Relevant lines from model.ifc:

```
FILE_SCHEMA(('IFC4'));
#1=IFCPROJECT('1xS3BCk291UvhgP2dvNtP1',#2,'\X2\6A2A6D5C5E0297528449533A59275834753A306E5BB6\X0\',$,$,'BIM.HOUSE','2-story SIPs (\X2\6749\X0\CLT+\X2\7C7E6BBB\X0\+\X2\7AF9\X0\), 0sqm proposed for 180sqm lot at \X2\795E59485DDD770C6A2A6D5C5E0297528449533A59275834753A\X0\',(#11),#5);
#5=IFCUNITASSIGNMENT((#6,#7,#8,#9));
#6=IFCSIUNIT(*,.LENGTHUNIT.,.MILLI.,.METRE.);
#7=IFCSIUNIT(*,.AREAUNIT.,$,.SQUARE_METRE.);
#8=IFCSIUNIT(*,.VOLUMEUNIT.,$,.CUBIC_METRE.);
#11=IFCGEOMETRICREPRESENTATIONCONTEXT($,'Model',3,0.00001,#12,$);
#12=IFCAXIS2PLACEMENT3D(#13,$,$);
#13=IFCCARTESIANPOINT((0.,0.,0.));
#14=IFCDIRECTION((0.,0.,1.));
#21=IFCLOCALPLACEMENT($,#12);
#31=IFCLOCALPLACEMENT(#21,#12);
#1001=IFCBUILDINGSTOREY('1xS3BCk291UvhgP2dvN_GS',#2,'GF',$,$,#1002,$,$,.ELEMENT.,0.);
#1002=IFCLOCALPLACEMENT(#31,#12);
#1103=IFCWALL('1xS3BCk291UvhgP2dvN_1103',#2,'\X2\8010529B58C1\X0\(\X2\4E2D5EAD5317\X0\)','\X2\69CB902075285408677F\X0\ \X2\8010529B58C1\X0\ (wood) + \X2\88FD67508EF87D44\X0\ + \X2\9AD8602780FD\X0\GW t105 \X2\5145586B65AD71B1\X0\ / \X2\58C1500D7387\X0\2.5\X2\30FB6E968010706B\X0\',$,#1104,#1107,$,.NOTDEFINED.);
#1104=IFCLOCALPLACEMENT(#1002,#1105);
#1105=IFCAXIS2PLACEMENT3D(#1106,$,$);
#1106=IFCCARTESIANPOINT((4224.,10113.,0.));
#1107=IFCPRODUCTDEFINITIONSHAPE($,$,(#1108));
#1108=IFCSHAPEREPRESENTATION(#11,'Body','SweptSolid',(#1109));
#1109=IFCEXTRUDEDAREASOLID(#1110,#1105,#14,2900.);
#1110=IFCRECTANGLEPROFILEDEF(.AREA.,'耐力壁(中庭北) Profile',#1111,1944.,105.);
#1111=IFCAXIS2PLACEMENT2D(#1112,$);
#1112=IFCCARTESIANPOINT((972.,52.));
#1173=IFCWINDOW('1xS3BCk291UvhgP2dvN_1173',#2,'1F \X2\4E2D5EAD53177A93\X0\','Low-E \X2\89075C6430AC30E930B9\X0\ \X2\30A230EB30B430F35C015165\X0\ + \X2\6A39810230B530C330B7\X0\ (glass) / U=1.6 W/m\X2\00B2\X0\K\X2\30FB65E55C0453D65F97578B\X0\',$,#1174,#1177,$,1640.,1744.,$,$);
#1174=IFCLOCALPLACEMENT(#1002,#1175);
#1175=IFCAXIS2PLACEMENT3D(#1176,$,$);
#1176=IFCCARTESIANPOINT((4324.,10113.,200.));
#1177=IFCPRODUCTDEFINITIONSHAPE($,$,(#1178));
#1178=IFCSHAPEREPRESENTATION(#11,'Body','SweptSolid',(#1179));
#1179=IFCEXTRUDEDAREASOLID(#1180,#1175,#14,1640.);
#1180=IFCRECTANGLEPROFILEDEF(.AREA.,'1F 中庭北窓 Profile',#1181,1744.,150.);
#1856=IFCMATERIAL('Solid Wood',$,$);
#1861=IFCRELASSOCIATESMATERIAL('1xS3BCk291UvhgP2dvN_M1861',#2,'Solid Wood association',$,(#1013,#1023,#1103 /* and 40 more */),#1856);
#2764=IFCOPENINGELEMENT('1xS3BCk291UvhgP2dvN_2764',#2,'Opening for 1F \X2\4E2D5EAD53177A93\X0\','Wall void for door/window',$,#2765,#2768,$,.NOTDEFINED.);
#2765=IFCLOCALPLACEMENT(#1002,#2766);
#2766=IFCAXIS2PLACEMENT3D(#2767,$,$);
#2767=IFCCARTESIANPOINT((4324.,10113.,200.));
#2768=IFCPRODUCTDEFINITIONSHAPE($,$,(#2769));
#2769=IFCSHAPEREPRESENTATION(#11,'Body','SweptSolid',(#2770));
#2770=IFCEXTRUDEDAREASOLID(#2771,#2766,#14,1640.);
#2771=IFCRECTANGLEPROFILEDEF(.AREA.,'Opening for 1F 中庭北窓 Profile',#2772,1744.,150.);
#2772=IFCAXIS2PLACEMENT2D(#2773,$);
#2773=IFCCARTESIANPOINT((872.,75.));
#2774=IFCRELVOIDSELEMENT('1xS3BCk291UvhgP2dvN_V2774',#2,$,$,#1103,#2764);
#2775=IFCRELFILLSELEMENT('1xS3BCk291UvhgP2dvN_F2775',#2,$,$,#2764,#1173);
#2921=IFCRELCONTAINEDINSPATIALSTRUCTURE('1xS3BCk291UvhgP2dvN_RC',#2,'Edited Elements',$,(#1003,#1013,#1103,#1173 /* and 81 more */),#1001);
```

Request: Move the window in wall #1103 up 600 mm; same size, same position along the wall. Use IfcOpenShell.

```python
import numpy as np
import ifcopenshell
import ifcopenshell.api.geometry
import ifcopenshell.util.placement
import ifcopenshell.util.unit

model = ifcopenshell.open("model.ifc")
unit_scale = ifcopenshell.util.unit.calculate_unit_scale(model)

window = model.by_guid("1xS3BCk291UvhgP2dvN_1173")
opening = window.FillsVoids[0].RelatingOpeningElement
dz = 0.6 / unit_scale

shift = np.array([0.0, 0.0, dz])
# The window is not placed relative to its opening, so move both.
for product in (opening, window):
    matrix = ifcopenshell.util.placement.get_local_placement(product.ObjectPlacement)
    matrix[:3, 3] += shift
    ifcopenshell.api.geometry.edit_object_placement(model, product=product, matrix=matrix, is_si=False)

print(f"moved by {dz * unit_scale:+.3f} m")

model.write("model_rev.ifc")
```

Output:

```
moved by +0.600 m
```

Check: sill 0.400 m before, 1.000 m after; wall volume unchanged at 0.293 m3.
